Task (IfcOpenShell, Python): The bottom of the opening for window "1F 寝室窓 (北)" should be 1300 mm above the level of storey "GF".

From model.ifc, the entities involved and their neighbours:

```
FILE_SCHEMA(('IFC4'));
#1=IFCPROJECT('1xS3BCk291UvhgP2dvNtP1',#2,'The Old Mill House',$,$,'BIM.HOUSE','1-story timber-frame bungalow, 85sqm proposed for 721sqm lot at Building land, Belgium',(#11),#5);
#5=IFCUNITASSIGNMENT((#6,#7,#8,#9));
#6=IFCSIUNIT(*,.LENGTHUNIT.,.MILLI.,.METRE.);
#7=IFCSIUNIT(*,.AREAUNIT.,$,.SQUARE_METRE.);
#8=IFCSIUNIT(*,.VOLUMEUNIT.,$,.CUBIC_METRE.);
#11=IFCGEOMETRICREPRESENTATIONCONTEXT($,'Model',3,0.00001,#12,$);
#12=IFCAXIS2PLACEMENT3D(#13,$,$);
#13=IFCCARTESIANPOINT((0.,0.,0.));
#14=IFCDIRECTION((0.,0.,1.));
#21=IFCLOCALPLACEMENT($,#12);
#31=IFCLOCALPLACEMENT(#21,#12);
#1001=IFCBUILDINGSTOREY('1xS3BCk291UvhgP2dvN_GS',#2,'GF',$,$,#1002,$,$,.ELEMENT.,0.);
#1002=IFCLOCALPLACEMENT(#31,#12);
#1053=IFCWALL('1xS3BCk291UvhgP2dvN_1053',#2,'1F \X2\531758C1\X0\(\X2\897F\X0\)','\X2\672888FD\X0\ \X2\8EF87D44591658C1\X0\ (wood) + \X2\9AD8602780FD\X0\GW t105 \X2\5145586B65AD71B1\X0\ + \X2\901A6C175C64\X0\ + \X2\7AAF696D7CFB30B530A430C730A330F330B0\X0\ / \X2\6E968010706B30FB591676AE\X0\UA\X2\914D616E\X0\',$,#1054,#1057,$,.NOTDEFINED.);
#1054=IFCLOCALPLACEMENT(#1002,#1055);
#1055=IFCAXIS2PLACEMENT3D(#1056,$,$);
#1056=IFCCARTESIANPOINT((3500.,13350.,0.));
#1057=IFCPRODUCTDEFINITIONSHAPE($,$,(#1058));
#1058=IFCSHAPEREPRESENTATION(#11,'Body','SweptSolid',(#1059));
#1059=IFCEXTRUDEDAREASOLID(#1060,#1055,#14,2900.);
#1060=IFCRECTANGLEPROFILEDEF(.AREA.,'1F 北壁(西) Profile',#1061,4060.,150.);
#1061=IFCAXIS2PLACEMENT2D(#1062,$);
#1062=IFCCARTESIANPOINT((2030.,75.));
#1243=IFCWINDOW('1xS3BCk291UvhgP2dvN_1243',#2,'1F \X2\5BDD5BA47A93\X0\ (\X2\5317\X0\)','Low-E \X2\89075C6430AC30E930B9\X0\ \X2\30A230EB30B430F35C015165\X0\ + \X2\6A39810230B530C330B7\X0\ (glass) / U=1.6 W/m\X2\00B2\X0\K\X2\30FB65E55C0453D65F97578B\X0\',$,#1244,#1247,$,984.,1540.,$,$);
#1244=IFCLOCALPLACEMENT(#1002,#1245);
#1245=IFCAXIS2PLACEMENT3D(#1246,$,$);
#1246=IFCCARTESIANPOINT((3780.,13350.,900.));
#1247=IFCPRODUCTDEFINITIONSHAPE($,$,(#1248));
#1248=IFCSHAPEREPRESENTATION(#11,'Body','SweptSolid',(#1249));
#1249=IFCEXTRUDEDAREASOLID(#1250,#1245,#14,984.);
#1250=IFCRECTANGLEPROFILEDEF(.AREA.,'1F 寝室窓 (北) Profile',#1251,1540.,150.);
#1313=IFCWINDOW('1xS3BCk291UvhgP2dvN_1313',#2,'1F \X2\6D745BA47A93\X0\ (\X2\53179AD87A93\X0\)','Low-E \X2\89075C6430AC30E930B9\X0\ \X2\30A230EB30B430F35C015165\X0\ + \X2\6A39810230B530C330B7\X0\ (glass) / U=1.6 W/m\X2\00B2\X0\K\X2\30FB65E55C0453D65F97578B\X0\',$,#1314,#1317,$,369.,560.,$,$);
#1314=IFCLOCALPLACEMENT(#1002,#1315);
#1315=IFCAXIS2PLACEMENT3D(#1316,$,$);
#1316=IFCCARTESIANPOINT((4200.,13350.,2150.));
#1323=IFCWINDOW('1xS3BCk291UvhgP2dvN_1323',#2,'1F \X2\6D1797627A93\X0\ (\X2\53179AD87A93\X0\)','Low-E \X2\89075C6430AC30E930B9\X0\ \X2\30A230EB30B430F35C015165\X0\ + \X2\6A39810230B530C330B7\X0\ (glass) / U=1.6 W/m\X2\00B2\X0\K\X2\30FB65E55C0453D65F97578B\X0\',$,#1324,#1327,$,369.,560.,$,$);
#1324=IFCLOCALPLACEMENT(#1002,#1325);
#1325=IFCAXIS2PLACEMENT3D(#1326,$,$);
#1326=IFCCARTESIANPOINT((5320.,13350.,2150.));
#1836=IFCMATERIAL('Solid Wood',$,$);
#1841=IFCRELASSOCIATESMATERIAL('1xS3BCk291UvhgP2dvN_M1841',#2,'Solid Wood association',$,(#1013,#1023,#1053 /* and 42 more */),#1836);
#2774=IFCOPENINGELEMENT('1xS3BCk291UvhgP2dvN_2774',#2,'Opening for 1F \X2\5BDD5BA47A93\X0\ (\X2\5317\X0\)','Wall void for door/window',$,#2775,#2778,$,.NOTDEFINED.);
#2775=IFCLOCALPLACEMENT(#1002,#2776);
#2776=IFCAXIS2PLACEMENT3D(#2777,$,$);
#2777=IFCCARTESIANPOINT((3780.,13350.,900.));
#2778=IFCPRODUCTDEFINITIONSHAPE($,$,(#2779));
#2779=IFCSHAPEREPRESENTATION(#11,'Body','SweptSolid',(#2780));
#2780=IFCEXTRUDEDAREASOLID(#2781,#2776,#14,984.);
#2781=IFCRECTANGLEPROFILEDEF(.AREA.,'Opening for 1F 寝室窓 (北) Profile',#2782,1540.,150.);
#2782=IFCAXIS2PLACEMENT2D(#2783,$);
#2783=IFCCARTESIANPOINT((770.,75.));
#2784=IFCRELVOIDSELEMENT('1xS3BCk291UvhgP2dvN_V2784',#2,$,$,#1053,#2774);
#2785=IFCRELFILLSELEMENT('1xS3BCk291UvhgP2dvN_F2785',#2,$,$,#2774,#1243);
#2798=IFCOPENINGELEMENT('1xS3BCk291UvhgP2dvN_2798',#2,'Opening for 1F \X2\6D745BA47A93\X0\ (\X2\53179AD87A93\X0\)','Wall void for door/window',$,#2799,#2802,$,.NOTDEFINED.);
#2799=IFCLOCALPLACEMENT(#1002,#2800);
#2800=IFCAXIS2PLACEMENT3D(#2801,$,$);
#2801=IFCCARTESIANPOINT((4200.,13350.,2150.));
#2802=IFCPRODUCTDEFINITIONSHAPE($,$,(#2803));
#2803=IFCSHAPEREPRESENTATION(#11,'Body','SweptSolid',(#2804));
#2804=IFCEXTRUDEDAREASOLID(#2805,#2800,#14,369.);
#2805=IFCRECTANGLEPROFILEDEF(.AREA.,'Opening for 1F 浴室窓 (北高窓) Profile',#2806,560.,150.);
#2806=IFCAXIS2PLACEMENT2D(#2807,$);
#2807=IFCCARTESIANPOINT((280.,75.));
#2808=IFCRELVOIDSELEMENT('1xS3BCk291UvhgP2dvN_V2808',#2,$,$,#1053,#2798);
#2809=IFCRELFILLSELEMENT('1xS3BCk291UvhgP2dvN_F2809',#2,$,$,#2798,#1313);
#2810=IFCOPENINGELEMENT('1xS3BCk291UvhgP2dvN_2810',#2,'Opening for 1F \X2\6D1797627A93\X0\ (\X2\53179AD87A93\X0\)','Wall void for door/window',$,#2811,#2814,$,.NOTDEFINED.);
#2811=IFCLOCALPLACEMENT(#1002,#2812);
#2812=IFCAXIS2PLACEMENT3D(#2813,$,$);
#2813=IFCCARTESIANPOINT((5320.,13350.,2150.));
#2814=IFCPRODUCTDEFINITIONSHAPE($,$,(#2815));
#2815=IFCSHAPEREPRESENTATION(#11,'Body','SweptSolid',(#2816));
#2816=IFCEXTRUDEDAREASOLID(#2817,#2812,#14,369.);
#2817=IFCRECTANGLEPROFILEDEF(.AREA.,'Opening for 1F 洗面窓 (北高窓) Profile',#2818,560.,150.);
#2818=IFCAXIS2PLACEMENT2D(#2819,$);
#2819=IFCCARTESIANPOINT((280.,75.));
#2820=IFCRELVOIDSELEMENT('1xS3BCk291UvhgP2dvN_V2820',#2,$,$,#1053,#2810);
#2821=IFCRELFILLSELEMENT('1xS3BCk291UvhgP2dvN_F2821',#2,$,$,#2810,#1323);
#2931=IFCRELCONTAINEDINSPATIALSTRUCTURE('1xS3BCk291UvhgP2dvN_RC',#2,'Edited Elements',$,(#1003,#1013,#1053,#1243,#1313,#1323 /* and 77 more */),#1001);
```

```python
import numpy as np
import ifcopenshell
import ifcopenshell.api.geometry
import ifcopenshell.geom
import ifcopenshell.util.element
import ifcopenshell.util.placement
import ifcopenshell.util.shape
import ifcopenshell.util.unit

model = ifcopenshell.open("model.ifc")
unit_scale = ifcopenshell.util.unit.calculate_unit_scale(model)

window = model.by_guid("1xS3BCk291UvhgP2dvN_1243")
opening = window.FillsVoids[0].RelatingOpeningElement
storey = ifcopenshell.util.element.get_container(window, ifc_class="IfcBuildingStorey")
level = ifcopenshell.util.placement.get_local_placement(storey.ObjectPlacement)[2, 3]

# The opening's origin need not be at the sill, so measure its lowest point.
shape = ifcopenshell.geom.create_shape(ifcopenshell.geom.settings(), opening)
bottom = ifcopenshell.util.shape.get_shape_bottom_elevation(shape, shape.geometry) / unit_scale
dz = level + 1.3 / unit_scale - bottom

shift = np.array([0.0, 0.0, dz])
# The window is not placed relative to its opening, so move both.
for product in (opening, window):
    matrix = ifcopenshell.util.placement.get_local_placement(product.ObjectPlacement)
    matrix[:3, 3] += shift
    ifcopenshell.api.geometry.edit_object_placement(model, product=product, matrix=matrix, is_si=False)

print(f"moved by {dz * unit_scale:+.3f} m")

model.write("model_rev.ifc")
```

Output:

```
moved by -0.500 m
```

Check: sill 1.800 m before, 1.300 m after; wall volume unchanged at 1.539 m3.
